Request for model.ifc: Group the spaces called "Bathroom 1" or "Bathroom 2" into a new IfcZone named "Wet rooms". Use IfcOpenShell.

First a look at what the model holds.

```python
import ifcopenshell

model = ifcopenshell.open("model.ifc")
print(model.schema)
seen = {}
for space in model.by_type("IfcSpace"):
    seen[space.LongName] = seen.get(space.LongName, 0) + 1
for name, count in sorted(seen.items(), key=str):
    print(count, "x", name)
print("zones:", [z.Name for z in model.by_type("IfcZone")][:20])
```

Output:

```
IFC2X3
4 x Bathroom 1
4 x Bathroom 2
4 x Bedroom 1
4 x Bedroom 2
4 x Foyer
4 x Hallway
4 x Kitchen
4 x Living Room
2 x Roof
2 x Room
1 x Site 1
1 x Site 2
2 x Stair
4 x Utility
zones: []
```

```python
import ifcopenshell
import ifcopenshell.api.group
import ifcopenshell.api.root

model = ifcopenshell.open("model.ifc")

names = {"Bathroom 1", "Bathroom 2"}
spaces = [s for s in model.by_type("IfcSpace") if s.LongName in names]

zone = ifcopenshell.api.root.create_entity(model, ifc_class="IfcZone", name="Wet rooms")
ifcopenshell.api.group.assign_group(model, products=spaces, group=zone)
print(len(spaces), "spaces in", zone.Name)

model.write("model-out.ifc")
```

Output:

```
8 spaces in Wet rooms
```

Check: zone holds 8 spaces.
